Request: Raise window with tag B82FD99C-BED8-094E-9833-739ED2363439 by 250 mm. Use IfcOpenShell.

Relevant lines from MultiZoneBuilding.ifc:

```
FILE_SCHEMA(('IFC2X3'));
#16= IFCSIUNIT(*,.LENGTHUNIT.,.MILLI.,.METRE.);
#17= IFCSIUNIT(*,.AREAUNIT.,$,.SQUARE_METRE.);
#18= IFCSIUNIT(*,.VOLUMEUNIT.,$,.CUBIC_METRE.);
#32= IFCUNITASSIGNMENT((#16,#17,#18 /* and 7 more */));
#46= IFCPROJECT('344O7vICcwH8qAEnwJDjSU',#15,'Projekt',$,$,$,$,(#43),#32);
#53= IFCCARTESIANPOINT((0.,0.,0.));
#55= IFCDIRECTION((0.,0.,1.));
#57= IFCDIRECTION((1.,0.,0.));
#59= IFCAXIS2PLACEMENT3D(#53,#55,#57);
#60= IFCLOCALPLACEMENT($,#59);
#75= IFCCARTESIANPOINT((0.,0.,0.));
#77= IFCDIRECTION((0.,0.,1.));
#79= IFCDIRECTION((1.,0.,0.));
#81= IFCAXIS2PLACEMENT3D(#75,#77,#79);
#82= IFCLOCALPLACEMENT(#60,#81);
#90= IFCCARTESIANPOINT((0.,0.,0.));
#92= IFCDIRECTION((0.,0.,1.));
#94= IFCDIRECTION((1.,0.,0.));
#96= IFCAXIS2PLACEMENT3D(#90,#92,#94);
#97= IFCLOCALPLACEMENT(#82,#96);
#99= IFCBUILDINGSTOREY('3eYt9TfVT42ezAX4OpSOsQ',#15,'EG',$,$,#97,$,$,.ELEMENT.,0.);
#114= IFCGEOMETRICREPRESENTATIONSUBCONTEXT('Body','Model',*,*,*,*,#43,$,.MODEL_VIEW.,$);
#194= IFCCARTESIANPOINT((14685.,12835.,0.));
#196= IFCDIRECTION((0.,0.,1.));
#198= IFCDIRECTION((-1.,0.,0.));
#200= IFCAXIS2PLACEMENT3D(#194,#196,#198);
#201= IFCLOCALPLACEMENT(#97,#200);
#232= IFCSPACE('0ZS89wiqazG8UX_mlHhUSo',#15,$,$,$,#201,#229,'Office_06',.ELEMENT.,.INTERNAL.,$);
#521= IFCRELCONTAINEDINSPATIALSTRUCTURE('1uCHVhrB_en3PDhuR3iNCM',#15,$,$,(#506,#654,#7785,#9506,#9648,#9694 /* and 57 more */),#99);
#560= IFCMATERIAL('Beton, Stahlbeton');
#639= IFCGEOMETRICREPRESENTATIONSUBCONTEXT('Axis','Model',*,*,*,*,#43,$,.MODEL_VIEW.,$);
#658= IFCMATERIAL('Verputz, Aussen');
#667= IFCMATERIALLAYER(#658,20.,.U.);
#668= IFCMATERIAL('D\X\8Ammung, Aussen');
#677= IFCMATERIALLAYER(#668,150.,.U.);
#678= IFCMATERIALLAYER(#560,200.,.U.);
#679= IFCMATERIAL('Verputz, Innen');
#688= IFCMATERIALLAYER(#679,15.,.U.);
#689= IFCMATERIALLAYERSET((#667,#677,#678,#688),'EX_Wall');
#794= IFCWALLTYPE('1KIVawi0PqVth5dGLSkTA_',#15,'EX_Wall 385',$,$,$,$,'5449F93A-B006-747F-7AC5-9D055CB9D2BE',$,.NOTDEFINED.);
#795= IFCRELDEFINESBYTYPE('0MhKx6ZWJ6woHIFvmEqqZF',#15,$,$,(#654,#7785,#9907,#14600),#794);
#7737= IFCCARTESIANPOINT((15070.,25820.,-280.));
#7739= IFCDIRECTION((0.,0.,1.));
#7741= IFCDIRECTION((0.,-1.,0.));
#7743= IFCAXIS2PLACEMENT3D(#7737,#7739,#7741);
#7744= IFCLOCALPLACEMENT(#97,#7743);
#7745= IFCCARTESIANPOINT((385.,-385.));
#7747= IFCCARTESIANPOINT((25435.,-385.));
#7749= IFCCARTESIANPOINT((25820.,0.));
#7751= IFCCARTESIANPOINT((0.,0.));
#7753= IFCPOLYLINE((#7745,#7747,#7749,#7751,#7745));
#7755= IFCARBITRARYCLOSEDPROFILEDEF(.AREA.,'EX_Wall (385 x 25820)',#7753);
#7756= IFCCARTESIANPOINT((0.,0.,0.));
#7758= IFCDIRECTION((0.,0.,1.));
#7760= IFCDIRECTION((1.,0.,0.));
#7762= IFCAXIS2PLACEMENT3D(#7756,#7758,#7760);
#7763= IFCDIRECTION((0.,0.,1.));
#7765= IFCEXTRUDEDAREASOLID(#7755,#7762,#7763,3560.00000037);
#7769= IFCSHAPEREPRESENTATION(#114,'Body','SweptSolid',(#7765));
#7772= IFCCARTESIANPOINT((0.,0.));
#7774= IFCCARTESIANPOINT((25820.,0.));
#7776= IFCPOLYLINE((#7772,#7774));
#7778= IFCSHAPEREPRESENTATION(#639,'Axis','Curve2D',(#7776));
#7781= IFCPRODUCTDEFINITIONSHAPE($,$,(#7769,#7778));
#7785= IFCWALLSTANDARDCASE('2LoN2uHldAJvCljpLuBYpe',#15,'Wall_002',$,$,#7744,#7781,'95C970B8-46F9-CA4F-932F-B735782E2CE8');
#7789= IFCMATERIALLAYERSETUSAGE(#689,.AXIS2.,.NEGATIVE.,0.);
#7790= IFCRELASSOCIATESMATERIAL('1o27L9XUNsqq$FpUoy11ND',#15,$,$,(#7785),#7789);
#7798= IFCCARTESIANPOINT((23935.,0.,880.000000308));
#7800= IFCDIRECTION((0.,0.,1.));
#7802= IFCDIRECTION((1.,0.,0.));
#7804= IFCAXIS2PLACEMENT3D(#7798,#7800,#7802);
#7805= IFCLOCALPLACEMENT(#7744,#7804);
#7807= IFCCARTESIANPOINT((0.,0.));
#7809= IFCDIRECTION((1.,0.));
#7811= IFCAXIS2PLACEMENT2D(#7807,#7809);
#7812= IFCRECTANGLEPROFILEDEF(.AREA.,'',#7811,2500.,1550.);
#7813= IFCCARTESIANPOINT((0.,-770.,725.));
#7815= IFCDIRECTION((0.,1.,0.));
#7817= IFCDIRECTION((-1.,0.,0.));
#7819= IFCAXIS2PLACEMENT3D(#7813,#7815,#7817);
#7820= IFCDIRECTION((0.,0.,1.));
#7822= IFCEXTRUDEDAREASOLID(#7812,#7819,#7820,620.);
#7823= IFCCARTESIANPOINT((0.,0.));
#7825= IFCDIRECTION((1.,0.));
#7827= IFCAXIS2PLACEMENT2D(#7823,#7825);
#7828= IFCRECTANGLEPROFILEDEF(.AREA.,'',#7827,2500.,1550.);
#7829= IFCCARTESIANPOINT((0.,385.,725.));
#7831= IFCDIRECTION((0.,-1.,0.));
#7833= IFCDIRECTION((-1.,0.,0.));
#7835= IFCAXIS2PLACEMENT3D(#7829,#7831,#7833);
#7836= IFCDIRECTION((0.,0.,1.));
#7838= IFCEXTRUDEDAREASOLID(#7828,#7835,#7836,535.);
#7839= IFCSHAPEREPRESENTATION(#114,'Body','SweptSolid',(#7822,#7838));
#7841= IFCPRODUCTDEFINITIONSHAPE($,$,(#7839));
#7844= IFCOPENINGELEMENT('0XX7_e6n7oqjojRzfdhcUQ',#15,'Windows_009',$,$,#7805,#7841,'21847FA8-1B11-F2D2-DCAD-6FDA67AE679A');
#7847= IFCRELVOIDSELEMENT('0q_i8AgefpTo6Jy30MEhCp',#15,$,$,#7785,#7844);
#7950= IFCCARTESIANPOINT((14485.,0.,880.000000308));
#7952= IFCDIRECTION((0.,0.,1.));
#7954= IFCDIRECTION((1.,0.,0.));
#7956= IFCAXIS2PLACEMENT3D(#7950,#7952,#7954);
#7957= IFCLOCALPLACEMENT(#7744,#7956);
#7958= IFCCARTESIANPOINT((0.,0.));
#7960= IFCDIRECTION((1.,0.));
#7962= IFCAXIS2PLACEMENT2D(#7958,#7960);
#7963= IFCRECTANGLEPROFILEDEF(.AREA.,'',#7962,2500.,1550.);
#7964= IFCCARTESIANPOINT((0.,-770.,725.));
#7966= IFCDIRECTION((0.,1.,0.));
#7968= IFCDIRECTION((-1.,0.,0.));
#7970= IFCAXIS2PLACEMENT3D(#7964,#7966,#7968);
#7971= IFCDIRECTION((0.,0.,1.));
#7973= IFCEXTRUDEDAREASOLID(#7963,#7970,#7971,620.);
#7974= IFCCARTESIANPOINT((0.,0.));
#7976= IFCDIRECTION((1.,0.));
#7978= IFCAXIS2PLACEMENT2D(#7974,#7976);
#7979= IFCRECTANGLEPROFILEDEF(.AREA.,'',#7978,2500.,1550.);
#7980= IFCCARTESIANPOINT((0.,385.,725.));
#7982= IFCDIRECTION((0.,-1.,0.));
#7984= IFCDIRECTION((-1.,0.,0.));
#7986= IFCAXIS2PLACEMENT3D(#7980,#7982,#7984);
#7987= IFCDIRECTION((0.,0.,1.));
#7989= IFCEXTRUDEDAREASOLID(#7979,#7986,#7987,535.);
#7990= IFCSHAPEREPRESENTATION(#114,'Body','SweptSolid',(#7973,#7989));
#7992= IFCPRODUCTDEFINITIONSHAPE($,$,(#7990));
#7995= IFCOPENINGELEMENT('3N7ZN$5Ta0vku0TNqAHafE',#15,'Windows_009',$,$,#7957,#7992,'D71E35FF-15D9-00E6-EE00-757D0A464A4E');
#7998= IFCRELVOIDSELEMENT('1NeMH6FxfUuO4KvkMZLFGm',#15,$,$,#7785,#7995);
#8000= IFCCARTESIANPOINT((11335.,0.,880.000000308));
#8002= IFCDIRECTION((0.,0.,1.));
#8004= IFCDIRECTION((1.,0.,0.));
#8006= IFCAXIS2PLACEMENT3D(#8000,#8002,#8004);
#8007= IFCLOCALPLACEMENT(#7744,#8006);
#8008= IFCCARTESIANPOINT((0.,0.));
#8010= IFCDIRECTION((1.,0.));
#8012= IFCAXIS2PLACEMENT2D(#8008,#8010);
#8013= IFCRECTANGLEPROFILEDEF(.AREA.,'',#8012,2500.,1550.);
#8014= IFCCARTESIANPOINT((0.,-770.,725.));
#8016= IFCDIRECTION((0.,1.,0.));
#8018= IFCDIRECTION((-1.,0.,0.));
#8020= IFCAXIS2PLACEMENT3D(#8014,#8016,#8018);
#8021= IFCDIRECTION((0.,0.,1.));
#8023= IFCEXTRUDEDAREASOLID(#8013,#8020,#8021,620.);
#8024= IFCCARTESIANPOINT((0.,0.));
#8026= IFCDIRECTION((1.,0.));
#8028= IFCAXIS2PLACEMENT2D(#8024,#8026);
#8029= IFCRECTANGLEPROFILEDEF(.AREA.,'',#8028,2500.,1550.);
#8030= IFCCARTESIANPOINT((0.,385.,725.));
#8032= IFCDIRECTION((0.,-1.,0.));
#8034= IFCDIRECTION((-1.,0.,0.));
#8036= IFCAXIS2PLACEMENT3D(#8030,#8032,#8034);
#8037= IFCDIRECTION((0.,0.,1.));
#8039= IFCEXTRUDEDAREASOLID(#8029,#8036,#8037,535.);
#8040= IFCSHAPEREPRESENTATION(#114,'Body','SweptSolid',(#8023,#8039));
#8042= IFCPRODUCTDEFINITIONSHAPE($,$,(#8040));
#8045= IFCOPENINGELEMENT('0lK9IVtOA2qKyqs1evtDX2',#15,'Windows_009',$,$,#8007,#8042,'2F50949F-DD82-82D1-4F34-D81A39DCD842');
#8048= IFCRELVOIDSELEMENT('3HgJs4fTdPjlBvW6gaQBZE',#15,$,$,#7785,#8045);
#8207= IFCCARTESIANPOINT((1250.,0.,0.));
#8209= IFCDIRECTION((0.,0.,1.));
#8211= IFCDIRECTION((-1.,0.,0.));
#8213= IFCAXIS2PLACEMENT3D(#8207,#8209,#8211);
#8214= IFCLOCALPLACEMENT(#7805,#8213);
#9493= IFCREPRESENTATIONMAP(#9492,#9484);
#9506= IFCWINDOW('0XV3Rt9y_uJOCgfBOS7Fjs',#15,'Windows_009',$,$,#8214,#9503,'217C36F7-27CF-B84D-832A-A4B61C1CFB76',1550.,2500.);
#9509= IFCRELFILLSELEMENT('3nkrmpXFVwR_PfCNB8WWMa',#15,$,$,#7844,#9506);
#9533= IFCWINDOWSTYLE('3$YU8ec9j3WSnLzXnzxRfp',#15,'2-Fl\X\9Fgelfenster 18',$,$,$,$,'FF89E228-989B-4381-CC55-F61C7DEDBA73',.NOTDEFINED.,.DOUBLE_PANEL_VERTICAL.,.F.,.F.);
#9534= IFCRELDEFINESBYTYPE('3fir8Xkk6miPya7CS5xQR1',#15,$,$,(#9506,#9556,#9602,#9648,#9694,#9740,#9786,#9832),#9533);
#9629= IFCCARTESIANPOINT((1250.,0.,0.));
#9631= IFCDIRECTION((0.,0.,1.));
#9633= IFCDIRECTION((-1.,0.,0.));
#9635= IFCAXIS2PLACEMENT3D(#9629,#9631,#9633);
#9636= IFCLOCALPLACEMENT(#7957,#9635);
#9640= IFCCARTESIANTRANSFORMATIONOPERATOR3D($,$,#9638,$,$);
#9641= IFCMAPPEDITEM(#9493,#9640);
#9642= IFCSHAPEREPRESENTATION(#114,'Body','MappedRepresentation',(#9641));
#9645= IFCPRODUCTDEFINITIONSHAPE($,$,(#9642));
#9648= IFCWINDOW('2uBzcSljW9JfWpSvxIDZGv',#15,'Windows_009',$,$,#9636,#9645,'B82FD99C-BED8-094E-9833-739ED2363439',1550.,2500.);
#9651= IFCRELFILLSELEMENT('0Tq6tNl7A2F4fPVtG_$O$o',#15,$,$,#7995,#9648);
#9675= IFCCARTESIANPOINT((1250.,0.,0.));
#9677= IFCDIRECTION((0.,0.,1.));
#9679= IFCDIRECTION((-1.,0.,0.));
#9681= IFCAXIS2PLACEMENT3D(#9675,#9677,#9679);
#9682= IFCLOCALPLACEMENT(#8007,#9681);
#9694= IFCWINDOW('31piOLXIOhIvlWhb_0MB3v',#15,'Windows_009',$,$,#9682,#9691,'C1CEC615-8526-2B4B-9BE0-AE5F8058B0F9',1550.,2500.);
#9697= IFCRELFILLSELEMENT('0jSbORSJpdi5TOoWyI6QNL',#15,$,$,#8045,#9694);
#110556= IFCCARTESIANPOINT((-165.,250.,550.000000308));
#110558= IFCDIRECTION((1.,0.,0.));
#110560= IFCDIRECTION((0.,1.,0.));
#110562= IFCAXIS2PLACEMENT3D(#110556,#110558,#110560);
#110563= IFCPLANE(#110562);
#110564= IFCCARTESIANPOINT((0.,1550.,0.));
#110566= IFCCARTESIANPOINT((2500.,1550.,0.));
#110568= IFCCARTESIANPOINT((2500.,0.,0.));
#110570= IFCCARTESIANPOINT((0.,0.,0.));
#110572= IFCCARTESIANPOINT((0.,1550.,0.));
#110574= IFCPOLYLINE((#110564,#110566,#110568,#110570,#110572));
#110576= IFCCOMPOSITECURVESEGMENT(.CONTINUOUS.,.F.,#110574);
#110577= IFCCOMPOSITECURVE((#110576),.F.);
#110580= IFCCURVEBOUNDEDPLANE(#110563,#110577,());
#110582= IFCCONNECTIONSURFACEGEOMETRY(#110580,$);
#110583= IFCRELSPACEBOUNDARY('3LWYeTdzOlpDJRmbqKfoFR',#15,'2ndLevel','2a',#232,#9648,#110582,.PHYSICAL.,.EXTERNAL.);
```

```python
import numpy as np
import ifcopenshell
import ifcopenshell.api.geometry
import ifcopenshell.util.placement
import ifcopenshell.util.unit

model = ifcopenshell.open("MultiZoneBuilding.ifc")
unit_scale = ifcopenshell.util.unit.calculate_unit_scale(model)

window = model.by_id(9648)
opening = window.FillsVoids[0].RelatingOpeningElement
dz = 0.25 / unit_scale

shift = np.array([0.0, 0.0, dz])
# The window is placed relative to its opening, so it follows when the opening moves.
matrix = ifcopenshell.util.placement.get_local_placement(opening.ObjectPlacement)
matrix[:3, 3] += shift
ifcopenshell.api.geometry.edit_object_placement(
    model, product=opening, matrix=matrix, is_si=False, should_transform_children=True
)

# Space boundary surfaces are stored in each space's coordinates; move them too.
for rel in window.ProvidesBoundaries:
    if not rel.ConnectionGeometry:
        continue
    surface = rel.ConnectionGeometry.SurfaceOnRelatingElement.BasisSurface
    space_matrix = ifcopenshell.util.placement.get_local_placement(rel.RelatingSpace.ObjectPlacement)
    point = np.array(surface.Position.Location.Coordinates) + space_matrix[:3, :3].T @ shift
    surface.Position = model.createIfcAxis2Placement3D(
        model.createIfcCartesianPoint(point.tolist()), surface.Position.Axis, surface.Position.RefDirection
    )

print(f"moved by {dz * unit_scale:+.3f} m")

model.write("MultiZoneBuilding_v2.ifc")
```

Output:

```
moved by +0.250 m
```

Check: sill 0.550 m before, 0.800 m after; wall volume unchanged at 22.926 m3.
